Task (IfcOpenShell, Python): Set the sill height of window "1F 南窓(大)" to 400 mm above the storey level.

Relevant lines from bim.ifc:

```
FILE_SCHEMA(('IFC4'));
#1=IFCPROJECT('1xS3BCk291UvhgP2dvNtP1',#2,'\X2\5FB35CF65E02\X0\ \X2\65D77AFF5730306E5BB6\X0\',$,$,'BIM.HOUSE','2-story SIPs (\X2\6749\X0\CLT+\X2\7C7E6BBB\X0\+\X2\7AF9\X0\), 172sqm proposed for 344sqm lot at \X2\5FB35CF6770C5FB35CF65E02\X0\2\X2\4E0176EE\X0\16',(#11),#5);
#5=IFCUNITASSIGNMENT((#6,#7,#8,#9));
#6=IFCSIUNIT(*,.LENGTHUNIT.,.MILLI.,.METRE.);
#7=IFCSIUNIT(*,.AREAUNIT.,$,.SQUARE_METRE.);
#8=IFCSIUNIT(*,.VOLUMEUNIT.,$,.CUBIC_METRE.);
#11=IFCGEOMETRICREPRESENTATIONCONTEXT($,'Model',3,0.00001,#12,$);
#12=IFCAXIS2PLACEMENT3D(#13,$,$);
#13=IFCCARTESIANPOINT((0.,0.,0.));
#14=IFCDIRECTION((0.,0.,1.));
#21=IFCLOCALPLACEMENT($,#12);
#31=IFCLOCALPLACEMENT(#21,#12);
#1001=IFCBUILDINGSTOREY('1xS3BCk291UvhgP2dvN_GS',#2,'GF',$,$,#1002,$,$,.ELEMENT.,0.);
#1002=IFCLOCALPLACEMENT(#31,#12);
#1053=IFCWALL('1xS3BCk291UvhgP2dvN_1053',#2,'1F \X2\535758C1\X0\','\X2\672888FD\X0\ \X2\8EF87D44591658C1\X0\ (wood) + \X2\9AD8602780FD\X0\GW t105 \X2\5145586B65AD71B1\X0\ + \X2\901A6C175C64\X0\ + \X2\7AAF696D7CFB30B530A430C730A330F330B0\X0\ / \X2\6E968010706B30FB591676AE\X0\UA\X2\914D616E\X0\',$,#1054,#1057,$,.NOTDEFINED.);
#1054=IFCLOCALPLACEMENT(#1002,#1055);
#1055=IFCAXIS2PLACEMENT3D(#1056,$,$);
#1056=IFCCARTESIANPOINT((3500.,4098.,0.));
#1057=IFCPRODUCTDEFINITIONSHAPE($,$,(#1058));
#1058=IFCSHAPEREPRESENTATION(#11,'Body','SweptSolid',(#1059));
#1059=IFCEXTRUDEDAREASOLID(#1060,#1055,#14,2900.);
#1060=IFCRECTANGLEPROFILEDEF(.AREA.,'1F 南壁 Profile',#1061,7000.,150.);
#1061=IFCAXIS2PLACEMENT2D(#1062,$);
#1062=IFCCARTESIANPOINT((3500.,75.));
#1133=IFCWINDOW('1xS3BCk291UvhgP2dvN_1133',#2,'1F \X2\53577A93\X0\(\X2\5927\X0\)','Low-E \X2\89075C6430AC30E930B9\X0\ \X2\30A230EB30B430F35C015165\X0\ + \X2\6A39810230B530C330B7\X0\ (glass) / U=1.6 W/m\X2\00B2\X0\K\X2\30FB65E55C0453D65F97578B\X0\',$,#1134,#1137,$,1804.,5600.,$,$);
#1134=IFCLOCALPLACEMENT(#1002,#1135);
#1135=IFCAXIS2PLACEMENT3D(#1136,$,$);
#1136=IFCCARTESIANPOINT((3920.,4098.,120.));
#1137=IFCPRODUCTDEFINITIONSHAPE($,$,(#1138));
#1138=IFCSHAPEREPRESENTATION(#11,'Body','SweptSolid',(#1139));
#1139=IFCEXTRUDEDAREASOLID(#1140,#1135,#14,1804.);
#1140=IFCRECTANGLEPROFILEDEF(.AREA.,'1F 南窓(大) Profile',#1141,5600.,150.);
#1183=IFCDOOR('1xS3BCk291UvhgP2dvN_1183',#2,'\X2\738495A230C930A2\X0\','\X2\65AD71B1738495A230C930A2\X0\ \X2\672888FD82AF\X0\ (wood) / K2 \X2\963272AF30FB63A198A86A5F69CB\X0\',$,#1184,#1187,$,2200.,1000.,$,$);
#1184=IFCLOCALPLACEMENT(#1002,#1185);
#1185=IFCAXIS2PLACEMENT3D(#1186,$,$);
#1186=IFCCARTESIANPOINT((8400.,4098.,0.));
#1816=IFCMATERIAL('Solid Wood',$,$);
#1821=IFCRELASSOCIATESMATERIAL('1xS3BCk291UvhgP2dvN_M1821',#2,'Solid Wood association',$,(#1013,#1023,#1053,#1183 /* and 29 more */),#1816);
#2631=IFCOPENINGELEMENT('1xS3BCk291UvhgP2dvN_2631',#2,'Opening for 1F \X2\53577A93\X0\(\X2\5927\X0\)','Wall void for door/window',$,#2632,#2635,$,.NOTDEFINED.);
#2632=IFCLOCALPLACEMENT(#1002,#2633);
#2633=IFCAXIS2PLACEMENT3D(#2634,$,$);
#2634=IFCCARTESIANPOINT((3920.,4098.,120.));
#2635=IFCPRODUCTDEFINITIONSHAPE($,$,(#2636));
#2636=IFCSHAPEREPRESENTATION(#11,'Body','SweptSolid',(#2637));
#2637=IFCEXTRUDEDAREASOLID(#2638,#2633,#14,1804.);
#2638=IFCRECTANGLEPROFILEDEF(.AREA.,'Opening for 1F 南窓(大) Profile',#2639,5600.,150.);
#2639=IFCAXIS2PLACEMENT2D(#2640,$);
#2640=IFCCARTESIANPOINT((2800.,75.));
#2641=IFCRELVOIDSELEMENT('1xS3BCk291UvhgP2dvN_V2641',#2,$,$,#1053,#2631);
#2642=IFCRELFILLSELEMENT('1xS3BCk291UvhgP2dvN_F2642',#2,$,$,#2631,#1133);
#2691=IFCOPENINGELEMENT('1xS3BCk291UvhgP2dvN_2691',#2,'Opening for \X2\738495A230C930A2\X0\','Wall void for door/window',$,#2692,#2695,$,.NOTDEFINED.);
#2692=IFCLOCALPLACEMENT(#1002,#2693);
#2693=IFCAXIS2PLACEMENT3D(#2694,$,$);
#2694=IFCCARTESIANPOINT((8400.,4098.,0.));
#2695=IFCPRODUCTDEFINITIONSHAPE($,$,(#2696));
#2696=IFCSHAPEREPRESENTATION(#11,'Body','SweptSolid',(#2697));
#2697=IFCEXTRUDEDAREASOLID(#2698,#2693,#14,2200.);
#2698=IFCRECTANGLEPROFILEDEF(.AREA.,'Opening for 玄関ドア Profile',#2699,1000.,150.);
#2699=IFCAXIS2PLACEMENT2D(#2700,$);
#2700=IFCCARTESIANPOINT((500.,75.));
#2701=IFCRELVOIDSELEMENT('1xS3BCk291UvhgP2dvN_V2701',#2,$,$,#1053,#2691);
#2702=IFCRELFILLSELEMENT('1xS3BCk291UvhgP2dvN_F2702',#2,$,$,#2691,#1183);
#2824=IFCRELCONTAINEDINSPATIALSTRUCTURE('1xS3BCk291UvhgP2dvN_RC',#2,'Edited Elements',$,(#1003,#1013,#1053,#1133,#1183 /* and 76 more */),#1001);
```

```python
import numpy as np
import ifcopenshell
import ifcopenshell.api.geometry
import ifcopenshell.geom
import ifcopenshell.util.element
import ifcopenshell.util.placement
import ifcopenshell.util.shape
import ifcopenshell.util.unit

model = ifcopenshell.open("bim.ifc")
unit_scale = ifcopenshell.util.unit.calculate_unit_scale(model)

window = model.by_guid("1xS3BCk291UvhgP2dvN_1133")
opening = window.FillsVoids[0].RelatingOpeningElement
storey = ifcopenshell.util.element.get_container(window, ifc_class="IfcBuildingStorey")
level = ifcopenshell.util.placement.get_local_placement(storey.ObjectPlacement)[2, 3]

# The opening's origin need not be at the sill, so measure its lowest point.
shape = ifcopenshell.geom.create_shape(ifcopenshell.geom.settings(), opening)
bottom = ifcopenshell.util.shape.get_shape_bottom_elevation(shape, shape.geometry) / unit_scale
dz = level + 0.4 / unit_scale - bottom

shift = np.array([0.0, 0.0, dz])
# The window is not placed relative to its opening, so move both.
for product in (opening, window):
    matrix = ifcopenshell.util.placement.get_local_placement(product.ObjectPlacement)
    matrix[:3, 3] += shift
    ifcopenshell.api.geometry.edit_object_placement(model, product=product, matrix=matrix, is_si=False)

print(f"moved by {dz * unit_scale:+.3f} m")

model.write("bim_v2.ifc")
```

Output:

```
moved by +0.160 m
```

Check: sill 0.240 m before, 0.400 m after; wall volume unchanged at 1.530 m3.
